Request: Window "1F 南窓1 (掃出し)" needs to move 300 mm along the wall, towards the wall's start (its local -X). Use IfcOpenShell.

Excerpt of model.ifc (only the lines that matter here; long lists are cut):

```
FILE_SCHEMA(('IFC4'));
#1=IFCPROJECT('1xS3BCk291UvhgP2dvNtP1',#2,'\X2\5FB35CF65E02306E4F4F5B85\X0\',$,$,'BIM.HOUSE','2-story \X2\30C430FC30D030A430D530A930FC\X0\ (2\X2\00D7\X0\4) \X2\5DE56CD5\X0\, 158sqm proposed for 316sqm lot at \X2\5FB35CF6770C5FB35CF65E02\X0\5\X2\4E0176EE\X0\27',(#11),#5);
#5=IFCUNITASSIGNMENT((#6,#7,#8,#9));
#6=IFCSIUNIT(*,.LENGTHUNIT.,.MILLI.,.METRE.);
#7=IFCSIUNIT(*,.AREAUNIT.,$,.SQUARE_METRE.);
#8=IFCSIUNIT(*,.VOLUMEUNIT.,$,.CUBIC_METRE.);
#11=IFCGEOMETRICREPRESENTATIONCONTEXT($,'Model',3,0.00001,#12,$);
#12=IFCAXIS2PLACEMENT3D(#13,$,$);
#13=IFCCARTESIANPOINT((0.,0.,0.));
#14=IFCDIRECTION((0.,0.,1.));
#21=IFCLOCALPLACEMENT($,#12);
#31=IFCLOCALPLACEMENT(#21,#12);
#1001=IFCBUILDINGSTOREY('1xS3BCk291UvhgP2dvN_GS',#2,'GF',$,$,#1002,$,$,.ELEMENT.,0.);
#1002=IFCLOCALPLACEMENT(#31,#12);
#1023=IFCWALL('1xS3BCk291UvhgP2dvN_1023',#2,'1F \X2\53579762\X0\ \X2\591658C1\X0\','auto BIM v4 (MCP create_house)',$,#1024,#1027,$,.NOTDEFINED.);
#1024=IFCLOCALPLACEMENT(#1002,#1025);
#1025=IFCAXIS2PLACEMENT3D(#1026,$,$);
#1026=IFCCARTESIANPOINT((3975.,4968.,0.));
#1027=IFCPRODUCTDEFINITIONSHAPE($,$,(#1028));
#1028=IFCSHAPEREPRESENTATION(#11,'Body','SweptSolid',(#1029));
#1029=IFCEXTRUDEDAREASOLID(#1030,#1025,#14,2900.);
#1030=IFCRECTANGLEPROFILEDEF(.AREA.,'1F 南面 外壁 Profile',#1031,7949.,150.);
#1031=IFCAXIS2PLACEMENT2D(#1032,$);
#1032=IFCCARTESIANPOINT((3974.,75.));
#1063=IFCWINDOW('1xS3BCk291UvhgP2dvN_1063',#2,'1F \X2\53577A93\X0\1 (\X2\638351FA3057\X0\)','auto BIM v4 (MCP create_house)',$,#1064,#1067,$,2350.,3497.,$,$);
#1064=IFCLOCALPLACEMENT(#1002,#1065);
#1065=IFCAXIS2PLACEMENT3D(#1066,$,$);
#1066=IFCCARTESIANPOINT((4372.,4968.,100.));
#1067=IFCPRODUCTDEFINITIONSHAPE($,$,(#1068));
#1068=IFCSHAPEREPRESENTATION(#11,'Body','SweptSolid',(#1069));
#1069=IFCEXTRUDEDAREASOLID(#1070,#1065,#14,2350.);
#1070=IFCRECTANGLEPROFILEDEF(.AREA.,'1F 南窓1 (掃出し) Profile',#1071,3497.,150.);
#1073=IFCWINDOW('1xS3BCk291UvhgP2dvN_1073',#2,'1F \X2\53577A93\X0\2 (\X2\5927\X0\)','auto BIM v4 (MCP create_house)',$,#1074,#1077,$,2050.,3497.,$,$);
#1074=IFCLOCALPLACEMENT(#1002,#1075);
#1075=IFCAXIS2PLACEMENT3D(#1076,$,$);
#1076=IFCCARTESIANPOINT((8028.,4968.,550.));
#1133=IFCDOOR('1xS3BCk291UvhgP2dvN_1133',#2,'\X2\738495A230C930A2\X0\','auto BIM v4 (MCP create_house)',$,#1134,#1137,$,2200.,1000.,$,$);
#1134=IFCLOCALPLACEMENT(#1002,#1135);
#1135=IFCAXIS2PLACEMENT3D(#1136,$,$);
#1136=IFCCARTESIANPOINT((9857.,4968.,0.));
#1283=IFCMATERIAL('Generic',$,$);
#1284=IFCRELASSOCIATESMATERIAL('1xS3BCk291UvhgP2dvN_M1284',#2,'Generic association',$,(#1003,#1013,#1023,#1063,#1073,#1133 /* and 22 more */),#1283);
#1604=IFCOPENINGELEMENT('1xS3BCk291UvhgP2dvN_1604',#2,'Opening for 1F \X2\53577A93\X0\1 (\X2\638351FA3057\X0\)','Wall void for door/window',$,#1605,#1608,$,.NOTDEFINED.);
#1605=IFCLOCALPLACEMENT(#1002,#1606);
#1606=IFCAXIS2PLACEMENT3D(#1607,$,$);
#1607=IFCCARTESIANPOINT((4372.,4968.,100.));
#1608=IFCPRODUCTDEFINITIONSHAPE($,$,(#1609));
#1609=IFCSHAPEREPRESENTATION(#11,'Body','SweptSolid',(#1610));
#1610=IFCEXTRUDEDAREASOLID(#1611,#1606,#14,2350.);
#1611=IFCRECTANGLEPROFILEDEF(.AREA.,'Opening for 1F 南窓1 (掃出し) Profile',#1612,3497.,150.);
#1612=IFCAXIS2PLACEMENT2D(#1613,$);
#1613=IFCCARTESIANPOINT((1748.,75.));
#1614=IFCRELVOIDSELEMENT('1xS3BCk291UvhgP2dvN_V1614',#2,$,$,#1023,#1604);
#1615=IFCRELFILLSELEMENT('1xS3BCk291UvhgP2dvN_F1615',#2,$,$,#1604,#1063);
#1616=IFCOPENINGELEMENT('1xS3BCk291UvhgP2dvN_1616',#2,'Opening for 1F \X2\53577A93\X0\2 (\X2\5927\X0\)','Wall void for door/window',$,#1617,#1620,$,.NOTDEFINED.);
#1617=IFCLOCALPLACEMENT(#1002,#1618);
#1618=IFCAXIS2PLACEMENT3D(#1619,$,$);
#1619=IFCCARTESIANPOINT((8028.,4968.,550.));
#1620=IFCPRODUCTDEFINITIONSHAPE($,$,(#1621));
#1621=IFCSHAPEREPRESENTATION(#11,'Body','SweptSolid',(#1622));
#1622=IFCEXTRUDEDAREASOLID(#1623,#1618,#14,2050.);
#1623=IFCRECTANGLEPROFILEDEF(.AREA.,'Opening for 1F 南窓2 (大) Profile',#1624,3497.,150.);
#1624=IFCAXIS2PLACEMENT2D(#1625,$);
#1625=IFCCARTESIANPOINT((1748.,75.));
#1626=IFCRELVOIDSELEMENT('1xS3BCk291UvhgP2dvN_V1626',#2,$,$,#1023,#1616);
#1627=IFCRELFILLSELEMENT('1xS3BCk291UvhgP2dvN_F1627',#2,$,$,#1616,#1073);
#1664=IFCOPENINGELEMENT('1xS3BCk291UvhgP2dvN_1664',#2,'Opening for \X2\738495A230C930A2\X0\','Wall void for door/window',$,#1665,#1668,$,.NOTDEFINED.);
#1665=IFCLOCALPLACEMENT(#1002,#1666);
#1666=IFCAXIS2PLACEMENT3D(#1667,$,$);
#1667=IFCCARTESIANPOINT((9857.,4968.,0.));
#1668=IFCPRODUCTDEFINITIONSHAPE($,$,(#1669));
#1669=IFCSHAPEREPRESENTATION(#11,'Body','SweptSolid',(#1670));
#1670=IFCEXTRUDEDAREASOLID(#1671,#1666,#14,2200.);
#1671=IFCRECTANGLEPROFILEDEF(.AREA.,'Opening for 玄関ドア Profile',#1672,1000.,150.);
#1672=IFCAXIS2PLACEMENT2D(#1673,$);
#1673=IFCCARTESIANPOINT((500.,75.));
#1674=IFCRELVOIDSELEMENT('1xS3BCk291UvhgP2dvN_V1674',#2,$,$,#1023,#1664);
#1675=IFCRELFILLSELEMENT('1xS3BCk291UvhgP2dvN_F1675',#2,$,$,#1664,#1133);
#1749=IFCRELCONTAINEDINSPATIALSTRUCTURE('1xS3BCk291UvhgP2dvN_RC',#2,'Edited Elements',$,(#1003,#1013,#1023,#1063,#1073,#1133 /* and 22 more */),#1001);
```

```python
import ifcopenshell
import ifcopenshell.api.geometry
import ifcopenshell.util.placement

model = ifcopenshell.open("model.ifc")

window = model.by_id(1063)
opening = window.FillsVoids[0].RelatingOpeningElement
wall = opening.VoidsElements[0].RelatingBuildingElement

wall_matrix = ifcopenshell.util.placement.get_local_placement(wall.ObjectPlacement)
shift = wall_matrix[:3, 0] * -300.0
before = ifcopenshell.util.placement.get_local_placement(window.ObjectPlacement)[:3, 3].copy()

# The window is not placed relative to its opening, so move both.
for product in (opening, window):
    matrix = ifcopenshell.util.placement.get_local_placement(product.ObjectPlacement)
    matrix[:3, 3] += shift
    ifcopenshell.api.geometry.edit_object_placement(model, product=product, matrix=matrix, is_si=False)

after = ifcopenshell.util.placement.get_local_placement(window.ObjectPlacement)[:3, 3]
print("window moved by", (after - before).round(3) + 0.0)

model.write("model-out.ifc")
```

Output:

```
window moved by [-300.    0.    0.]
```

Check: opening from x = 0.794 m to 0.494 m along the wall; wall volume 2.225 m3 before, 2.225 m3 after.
